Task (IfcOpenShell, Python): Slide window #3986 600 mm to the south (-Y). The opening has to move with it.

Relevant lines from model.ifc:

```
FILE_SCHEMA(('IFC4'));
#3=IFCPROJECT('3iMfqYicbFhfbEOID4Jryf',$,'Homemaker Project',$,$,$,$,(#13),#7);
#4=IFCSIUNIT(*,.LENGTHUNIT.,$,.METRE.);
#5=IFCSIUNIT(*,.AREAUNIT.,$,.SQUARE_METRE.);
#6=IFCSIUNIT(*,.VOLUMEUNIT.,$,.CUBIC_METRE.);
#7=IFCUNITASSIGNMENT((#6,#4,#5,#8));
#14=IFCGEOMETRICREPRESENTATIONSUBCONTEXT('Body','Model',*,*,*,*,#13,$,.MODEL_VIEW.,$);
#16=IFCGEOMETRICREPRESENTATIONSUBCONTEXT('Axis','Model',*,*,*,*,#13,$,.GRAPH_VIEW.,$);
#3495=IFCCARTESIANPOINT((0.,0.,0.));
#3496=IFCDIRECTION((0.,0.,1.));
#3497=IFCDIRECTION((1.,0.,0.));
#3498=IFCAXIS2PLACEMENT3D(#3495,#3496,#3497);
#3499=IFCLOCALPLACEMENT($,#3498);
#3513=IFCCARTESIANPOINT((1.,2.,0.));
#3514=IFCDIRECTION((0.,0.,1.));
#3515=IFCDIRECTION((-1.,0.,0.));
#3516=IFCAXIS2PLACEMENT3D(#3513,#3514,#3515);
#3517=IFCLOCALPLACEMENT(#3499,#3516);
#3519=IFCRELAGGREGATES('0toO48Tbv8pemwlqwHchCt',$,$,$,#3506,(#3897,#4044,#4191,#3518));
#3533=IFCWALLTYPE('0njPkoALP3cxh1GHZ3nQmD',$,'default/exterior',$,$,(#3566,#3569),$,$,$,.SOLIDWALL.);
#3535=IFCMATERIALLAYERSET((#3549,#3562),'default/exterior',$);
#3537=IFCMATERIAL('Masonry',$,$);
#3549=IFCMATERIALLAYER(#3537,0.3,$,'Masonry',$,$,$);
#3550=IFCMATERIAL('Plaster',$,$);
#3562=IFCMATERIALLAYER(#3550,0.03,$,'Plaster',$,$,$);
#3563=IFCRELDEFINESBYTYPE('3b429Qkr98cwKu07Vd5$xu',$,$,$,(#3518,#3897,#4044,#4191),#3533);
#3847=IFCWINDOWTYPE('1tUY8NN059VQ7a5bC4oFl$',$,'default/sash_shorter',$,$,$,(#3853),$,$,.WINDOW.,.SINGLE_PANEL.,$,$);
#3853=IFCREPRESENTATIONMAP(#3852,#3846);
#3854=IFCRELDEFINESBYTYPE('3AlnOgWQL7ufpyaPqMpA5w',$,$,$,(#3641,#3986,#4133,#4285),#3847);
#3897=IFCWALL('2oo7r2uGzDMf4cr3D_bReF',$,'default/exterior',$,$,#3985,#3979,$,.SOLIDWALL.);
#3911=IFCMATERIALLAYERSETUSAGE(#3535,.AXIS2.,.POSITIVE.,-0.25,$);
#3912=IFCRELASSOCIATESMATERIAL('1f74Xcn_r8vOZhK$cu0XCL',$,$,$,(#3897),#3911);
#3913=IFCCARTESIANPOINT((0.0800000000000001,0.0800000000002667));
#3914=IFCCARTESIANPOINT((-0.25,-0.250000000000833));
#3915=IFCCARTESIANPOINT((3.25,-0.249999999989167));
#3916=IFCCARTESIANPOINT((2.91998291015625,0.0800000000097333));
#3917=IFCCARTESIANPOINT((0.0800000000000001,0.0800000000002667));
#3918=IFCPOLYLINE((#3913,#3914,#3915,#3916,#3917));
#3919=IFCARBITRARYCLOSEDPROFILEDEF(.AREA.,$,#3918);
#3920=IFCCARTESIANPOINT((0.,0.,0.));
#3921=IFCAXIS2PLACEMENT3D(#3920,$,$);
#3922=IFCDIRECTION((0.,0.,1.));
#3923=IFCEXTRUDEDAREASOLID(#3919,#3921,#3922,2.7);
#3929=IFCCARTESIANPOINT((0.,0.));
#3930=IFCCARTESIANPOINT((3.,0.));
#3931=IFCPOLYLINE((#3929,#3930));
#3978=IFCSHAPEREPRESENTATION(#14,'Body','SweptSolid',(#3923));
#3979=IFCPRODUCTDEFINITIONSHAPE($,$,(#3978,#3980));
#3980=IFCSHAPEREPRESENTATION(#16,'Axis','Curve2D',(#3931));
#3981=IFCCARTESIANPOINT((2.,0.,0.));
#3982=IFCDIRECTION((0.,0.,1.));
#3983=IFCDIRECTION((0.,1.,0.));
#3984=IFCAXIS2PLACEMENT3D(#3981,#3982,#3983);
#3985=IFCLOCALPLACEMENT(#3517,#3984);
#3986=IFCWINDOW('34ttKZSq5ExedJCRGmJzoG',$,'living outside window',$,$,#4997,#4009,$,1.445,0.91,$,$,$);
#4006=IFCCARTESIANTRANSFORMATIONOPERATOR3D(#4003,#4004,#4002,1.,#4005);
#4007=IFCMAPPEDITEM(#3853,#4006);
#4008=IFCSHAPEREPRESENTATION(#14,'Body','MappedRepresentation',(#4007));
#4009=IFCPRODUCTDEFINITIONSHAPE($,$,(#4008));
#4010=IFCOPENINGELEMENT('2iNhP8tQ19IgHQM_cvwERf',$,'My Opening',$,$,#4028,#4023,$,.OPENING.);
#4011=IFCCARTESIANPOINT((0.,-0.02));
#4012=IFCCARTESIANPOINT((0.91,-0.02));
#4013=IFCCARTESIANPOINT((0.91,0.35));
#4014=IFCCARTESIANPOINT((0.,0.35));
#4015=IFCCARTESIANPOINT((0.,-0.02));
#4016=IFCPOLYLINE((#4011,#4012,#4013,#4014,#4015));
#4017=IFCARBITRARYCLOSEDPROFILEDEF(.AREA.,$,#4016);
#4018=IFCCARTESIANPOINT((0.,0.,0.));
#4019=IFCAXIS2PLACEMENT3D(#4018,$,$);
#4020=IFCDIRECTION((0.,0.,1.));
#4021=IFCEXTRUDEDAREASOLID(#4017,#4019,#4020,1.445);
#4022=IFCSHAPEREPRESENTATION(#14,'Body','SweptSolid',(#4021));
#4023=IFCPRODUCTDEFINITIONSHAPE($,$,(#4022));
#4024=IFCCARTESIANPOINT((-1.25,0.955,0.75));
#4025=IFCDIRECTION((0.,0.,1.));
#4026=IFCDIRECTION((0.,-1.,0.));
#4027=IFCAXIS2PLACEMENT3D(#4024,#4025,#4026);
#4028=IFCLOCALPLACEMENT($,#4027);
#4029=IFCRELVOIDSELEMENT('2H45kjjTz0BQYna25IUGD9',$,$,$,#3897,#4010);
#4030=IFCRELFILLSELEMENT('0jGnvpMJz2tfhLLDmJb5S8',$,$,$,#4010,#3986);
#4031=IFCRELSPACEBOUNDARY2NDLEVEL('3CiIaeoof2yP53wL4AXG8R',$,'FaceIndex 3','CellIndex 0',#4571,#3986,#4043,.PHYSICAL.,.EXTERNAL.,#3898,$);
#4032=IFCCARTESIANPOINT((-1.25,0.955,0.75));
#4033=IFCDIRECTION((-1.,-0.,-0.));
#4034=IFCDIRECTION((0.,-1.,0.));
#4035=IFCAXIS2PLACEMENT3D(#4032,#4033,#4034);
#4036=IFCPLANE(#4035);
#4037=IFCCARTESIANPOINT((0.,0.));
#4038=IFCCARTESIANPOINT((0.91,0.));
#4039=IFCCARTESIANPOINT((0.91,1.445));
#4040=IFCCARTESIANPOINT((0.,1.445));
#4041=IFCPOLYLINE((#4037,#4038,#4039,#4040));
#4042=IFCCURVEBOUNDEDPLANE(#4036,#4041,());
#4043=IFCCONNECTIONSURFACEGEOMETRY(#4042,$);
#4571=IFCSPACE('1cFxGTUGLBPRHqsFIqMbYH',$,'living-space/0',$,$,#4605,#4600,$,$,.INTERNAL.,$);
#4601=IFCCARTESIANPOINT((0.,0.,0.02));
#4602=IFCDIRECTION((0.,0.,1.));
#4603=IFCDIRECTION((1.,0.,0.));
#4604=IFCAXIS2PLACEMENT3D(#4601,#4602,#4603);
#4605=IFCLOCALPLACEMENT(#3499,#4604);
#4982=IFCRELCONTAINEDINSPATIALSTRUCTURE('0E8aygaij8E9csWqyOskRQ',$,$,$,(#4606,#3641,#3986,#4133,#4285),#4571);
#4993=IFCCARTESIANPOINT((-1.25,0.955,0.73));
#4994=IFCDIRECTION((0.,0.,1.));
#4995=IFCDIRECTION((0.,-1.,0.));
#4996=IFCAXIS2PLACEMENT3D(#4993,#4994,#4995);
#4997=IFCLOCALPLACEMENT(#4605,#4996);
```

```python
import numpy as np
import ifcopenshell
import ifcopenshell.api.geometry
import ifcopenshell.util.placement

model = ifcopenshell.open("model.ifc")

window = model.by_guid("34ttKZSq5ExedJCRGmJzoG")
opening = window.FillsVoids[0].RelatingOpeningElement
wall = opening.VoidsElements[0].RelatingBuildingElement

wall_matrix = ifcopenshell.util.placement.get_local_placement(wall.ObjectPlacement)
shift = wall_matrix[:3, 0] * 0.6
before = ifcopenshell.util.placement.get_local_placement(window.ObjectPlacement)[:3, 3].copy()

# The window is not placed relative to its opening, so move both.
for product in (opening, window):
    matrix = ifcopenshell.util.placement.get_local_placement(product.ObjectPlacement)
    matrix[:3, 3] += shift
    ifcopenshell.api.geometry.edit_object_placement(model, product=product, matrix=matrix, is_si=False)

# Space boundary surfaces are stored in each space's coordinates; move them too.
for rel in window.ProvidesBoundaries:
    if not rel.ConnectionGeometry:
        continue
    surface = rel.ConnectionGeometry.SurfaceOnRelatingElement.BasisSurface
    space_matrix = ifcopenshell.util.placement.get_local_placement(rel.RelatingSpace.ObjectPlacement)
    point = np.array(surface.Position.Location.Coordinates) + space_matrix[:3, :3].T @ shift
    surface.Position = model.createIfcAxis2Placement3D(
        model.createIfcCartesianPoint(point.tolist()), surface.Position.Axis, surface.Position.RefDirection
    )

after = ifcopenshell.util.placement.get_local_placement(window.ObjectPlacement)[:3, 3]
print("window moved by", (after - before).round(3) + 0.0)

model.write("model_updated.ifc")
```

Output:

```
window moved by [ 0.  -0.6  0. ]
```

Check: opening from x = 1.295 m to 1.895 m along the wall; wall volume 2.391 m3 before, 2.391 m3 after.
